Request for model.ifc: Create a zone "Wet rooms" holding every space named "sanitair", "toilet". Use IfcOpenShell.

First a look at what the model holds.

```python
import ifcopenshell

model = ifcopenshell.open("model.ifc")
print(model.schema)
seen = {}
for space in model.by_type("IfcSpace"):
    seen[space.LongName] = seen.get(space.LongName, 0) + 1
for name, count in sorted(seen.items(), key=str):
    print(count, "x", name)
print("zones:", [z.Name for z in model.by_type("IfcZone")][:20])
```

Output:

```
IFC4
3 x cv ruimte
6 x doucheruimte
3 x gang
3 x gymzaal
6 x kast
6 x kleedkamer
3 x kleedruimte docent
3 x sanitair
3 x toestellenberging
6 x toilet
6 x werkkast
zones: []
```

```python
import ifcopenshell
import ifcopenshell.api.group
import ifcopenshell.api.root

model = ifcopenshell.open("model.ifc")

names = {"sanitair", "toilet"}
spaces = [s for s in model.by_type("IfcSpace") if s.LongName in names]

zone = ifcopenshell.api.root.create_entity(model, ifc_class="IfcZone", name="Wet rooms")
ifcopenshell.api.group.assign_group(model, products=spaces, group=zone)
print(len(spaces), "spaces in", zone.Name)

model.write("model_updated.ifc")
```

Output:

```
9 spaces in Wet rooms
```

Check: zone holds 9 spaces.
